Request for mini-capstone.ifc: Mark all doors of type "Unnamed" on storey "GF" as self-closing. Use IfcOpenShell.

First a look at what the model holds.

```python
import ifcopenshell
import ifcopenshell.util.element

model = ifcopenshell.open("mini-capstone.ifc")
print(model.schema)
storey = next(s for s in model.by_type("IfcBuildingStorey") if s.Name == "GF")
doors = [e for e in ifcopenshell.util.element.get_decomposition(storey) if e.is_a("IfcDoor")]
seen = {}
for e in doors:
    element_type = ifcopenshell.util.element.get_type(e)
    key = (element_type.Name if element_type != e and element_type else None, ifcopenshell.util.element.get_pset(e, "Pset_DoorCommon", "SelfClosing"))
    seen[key] = seen.get(key, 0) + 1
for (name, value), count in sorted(seen.items(), key=str):
    print(count, "x", name, "|", value)
```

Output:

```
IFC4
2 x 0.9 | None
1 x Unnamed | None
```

```python
import ifcopenshell
import ifcopenshell.api.pset
import ifcopenshell.util.element

model = ifcopenshell.open("mini-capstone.ifc")

storey = next(s for s in model.by_type("IfcBuildingStorey") if s.Name == "GF")
doors = [e for e in ifcopenshell.util.element.get_decomposition(storey) if e.is_a("IfcDoor")]

count = 0
for e in doors:
    element_type = ifcopenshell.util.element.get_type(e)
    if element_type in (None, e) or element_type.Name != "Unnamed":
        continue
    # add_pset returns the element's existing set when there is one.
    pset = ifcopenshell.api.pset.add_pset(model, product=e, name="Pset_DoorCommon")
    ifcopenshell.api.pset.edit_pset(model, pset=pset, properties={"SelfClosing": True})
    count += 1

print(count, "doors updated")

model.write("mini-capstone-out.ifc")
```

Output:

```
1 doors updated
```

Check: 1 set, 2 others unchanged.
